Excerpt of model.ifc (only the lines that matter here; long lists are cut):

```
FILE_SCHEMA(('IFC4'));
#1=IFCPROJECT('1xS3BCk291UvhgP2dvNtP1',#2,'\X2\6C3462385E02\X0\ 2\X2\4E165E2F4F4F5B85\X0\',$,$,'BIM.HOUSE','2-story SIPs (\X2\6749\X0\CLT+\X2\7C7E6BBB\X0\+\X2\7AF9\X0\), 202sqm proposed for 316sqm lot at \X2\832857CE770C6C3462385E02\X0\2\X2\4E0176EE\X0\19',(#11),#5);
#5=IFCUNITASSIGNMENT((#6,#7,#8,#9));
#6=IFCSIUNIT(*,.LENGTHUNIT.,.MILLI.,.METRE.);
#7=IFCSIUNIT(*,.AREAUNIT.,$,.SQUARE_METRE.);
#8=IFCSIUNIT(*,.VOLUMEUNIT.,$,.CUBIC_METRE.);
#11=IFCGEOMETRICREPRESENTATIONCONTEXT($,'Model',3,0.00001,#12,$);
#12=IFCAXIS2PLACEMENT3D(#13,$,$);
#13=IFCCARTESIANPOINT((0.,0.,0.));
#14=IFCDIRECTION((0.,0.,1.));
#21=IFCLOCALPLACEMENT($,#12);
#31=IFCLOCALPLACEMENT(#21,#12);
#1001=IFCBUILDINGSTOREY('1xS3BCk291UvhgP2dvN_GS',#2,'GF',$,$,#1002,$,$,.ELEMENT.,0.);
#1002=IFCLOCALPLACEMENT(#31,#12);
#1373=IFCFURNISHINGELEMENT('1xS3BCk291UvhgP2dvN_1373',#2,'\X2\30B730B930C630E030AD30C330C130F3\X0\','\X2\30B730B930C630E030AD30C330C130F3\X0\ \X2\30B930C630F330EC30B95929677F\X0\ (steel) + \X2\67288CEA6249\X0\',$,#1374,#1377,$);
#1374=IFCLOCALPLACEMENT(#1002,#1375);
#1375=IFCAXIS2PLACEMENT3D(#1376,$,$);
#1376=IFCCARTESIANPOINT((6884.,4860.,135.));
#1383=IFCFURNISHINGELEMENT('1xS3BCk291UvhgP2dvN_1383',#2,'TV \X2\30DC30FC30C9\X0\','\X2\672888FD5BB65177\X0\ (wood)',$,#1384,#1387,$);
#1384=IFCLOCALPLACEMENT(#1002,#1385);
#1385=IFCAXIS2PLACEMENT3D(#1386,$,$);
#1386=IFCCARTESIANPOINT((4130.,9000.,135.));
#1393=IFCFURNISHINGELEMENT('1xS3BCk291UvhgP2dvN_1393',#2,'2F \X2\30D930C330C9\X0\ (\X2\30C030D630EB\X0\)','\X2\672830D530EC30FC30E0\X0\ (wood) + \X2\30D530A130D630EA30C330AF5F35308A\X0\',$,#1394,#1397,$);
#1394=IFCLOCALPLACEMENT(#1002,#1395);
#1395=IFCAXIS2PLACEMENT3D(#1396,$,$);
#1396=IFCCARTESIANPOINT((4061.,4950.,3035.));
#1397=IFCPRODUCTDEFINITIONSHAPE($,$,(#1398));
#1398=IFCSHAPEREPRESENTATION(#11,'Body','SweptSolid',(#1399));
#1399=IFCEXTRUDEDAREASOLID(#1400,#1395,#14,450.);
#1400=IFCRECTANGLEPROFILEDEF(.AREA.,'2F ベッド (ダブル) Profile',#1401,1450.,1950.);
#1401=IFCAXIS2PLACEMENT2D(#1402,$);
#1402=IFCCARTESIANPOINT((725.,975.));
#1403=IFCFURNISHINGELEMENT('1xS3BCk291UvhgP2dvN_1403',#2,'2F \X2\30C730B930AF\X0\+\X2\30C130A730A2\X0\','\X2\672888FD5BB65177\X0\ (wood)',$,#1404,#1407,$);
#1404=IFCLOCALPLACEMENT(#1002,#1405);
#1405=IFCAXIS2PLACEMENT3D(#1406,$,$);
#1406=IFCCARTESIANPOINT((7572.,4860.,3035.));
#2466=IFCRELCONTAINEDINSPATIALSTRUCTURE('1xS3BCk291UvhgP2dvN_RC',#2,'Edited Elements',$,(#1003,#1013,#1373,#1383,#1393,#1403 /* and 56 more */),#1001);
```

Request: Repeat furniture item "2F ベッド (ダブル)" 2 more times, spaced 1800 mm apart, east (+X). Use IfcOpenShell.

```python
import numpy as np
import ifcopenshell
import ifcopenshell.api.geometry
import ifcopenshell.api.root
import ifcopenshell.util.element
import ifcopenshell.util.placement

model = ifcopenshell.open("model.ifc")


def reuse_history(source, copy):
    """copy_class also copies each property set's owner history, people and application; keep the originals."""
    for rel in copy.IsDefinedBy:
        if rel.is_a("IfcRelDefinesByProperties") and (history := rel.RelatingPropertyDefinition.OwnerHistory):
            rel.RelatingPropertyDefinition.OwnerHistory = source.OwnerHistory
            ifcopenshell.util.element.remove_deep2(model, history)


source = model.by_id(1393)
base = ifcopenshell.util.placement.get_local_placement(source.ObjectPlacement)
step = np.array([1.0, 0.0, 0.0]) * 1800.0

for i in range(1, 3):
    copy = ifcopenshell.api.root.copy_class(model, product=source)
    copy.Representation = ifcopenshell.util.element.copy_deep(
        model, source.Representation, exclude=["IfcGeometricRepresentationContext", "IfcRepresentationMap"]
    )
    reuse_history(source, copy)
    matrix = base.copy()
    matrix[:3, 3] += i * step
    print("added at", matrix[:3, 3].round(3) + 0.0)
    ifcopenshell.api.geometry.edit_object_placement(model, product=copy, matrix=matrix, is_si=False)

model.write("model-out.ifc")
```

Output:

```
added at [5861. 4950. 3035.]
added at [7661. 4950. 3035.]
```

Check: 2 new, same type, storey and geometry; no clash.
